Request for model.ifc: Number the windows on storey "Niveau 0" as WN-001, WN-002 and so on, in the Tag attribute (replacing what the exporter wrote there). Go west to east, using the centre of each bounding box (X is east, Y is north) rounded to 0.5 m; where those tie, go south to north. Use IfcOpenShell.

First a look at what the model holds.

```python
import ifcopenshell
import ifcopenshell.util.element
import ifcopenshell.util.placement

model = ifcopenshell.open("model.ifc")
print(model.schema)
storey = next(s for s in model.by_type("IfcBuildingStorey") if s.Name == "Niveau 0")
windows = [e for e in ifcopenshell.util.element.get_decomposition(storey) if e.is_a("IfcWindow")]
for e in sorted(windows, key=lambda e: e.id()):
    origin = ifcopenshell.util.placement.get_local_placement(e.ObjectPlacement)[:3, 3]
    print(e.id(), e.Tag, e.Name, origin.round(2) + 0.0, sep=" | ")
```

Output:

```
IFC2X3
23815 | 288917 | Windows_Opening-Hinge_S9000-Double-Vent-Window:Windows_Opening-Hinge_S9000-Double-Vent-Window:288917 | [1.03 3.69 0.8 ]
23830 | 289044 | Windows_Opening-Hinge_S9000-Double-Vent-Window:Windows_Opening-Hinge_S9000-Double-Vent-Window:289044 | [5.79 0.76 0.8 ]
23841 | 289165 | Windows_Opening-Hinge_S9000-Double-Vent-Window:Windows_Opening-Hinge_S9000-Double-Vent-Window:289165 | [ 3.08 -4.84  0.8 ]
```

```python
import ifcopenshell
import ifcopenshell.geom
import ifcopenshell.util.element
import ifcopenshell.util.shape

model = ifcopenshell.open("model.ifc")
settings = ifcopenshell.geom.settings()
settings.set("use-world-coords", True)


def centre(element):
    shape = ifcopenshell.geom.create_shape(settings, element)
    return ifcopenshell.util.shape.get_bbox_centroid(shape.geometry)


storey = next(s for s in model.by_type("IfcBuildingStorey") if s.Name == "Niveau 0")
windows = [e for e in ifcopenshell.util.element.get_decomposition(storey) if e.is_a("IfcWindow")]

# Insertion points can sit at a corner or the storey origin, so sort by the geometry (in metres).
centres = {e: centre(e) for e in windows}
windows.sort(key=lambda e: (round(centres[e][0] / 0.5), centres[e][1]))

for i, e in enumerate(windows, start=1):
    number = f"WN-0{i:02d}"
    e.Tag = number
    print(e.id(), number)

model.write("model_updated.ifc")
```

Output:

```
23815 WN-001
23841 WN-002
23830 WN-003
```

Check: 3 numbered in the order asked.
